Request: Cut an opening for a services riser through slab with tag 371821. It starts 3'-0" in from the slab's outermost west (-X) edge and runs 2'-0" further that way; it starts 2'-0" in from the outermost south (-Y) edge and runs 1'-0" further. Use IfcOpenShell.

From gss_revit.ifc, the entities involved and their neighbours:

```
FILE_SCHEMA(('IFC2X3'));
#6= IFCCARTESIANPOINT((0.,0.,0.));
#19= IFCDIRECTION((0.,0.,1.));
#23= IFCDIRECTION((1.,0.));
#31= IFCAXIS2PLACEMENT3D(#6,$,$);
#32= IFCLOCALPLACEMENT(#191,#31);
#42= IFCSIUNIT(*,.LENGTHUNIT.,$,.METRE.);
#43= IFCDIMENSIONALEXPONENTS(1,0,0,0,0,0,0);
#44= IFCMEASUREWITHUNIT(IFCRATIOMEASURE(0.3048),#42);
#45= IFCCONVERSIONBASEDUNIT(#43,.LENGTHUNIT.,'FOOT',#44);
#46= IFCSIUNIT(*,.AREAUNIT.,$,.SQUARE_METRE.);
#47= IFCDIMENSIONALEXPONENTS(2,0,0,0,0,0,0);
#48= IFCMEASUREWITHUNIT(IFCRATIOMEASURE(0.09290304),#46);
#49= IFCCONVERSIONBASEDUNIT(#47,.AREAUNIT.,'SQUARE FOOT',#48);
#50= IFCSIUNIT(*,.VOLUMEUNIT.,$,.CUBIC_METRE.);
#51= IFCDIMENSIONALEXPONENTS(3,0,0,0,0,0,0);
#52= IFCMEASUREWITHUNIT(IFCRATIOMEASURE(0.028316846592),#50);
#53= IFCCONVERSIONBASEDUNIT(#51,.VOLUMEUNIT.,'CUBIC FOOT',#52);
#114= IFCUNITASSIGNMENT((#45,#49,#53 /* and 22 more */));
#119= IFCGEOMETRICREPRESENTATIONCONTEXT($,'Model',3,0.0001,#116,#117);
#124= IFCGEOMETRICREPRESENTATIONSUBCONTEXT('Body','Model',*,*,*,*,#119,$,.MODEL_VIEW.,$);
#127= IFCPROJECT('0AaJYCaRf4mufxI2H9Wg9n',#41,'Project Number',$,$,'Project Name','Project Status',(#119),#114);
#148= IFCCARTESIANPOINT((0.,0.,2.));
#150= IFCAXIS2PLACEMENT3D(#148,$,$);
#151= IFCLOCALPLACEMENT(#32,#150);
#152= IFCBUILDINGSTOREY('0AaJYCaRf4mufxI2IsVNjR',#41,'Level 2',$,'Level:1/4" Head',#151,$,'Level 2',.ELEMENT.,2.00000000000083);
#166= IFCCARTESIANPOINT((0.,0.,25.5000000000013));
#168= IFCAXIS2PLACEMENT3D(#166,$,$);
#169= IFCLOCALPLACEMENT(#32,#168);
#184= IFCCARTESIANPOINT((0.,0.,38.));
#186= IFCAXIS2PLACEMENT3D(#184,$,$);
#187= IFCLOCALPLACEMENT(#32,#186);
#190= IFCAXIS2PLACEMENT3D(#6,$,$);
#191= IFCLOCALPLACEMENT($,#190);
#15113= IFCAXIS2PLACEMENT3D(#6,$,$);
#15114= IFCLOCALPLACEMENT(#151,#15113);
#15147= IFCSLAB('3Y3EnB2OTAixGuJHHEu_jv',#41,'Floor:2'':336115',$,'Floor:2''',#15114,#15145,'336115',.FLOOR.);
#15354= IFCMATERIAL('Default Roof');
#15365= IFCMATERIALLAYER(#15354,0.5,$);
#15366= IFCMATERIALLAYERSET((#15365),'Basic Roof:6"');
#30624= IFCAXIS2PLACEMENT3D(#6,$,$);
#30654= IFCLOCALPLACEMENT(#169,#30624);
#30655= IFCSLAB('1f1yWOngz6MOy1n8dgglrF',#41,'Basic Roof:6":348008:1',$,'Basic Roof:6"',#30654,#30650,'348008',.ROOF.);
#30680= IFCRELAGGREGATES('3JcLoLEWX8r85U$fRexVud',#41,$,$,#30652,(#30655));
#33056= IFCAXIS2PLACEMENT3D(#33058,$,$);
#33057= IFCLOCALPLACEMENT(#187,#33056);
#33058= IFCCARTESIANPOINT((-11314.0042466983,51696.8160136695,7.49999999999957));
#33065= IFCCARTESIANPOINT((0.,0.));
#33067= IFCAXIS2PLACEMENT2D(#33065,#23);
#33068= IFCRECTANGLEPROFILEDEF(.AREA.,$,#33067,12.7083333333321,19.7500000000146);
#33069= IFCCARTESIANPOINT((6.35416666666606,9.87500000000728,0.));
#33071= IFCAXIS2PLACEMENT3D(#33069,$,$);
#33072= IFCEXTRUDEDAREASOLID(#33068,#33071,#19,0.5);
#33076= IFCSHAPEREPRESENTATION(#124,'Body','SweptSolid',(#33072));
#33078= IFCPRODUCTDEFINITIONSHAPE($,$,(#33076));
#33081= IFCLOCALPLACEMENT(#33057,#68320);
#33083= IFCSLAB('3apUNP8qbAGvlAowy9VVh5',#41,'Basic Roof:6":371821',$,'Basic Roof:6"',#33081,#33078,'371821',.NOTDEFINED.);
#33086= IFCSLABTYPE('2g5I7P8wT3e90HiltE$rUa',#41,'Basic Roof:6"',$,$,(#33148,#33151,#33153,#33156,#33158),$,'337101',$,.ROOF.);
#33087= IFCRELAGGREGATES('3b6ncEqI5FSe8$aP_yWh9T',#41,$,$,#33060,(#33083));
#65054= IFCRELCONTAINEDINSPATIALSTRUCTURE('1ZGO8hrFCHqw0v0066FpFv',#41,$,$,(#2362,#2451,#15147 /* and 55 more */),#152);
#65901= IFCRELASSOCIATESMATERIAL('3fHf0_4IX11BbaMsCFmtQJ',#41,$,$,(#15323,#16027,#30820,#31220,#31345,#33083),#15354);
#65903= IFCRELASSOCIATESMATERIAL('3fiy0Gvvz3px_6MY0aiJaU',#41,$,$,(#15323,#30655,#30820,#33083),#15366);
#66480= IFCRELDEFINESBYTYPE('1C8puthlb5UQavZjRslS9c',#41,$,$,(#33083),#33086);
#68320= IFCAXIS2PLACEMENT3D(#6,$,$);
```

```python
import numpy as np
import ifcopenshell
import ifcopenshell.api.feature
import ifcopenshell.api.geometry
import ifcopenshell.api.root
import ifcopenshell.geom
import ifcopenshell.util.placement
import ifcopenshell.util.representation
import ifcopenshell.util.shape
import ifcopenshell.util.unit

model = ifcopenshell.open("gss_revit.ifc")
unit_scale = ifcopenshell.util.unit.calculate_unit_scale(model)
settings = ifcopenshell.geom.settings()


def volume(element):
    """Net volume in cubic metres, openings subtracted."""
    shape = ifcopenshell.geom.create_shape(settings, element)
    return ifcopenshell.util.shape.get_volume(shape.geometry)


slab = model.by_guid("3apUNP8qbAGvlAowy9VVh5")
before = volume(slab)

# Extent in the slab's own axes, in metres. The edges named are its -X and -Y sides.
slab_shape = ifcopenshell.geom.create_shape(settings, slab)
vertices = ifcopenshell.util.shape.get_vertices(slab_shape.geometry)
x_min, y_min, bottom = vertices.min(axis=0)
top = vertices[:, 2].max()

opening = ifcopenshell.api.root.create_entity(model, ifc_class="IfcOpeningElement", name="Services riser opening")
context = ifcopenshell.util.representation.get_context(model, "Model", "Body", "MODEL_VIEW")
width, depth = 0.6096, 0.3048
outline = [(0.0, 0.0), (width, 0.0), (width, depth), (0.0, depth), (0.0, 0.0)]
# Overshoot both faces by 50 mm so the cut is clean.
shape = ifcopenshell.api.geometry.add_slab_representation(
    model, context=context, depth=top - bottom + 0.1, polyline=outline
)
ifcopenshell.api.geometry.assign_representation(model, product=opening, representation=shape)

matrix = ifcopenshell.util.placement.get_local_placement(slab.ObjectPlacement)
matrix[:, 3] = matrix @ np.append(np.array([x_min + 0.9144, y_min + 0.6096, bottom - 0.05]) / unit_scale, 1.0)
ifcopenshell.api.geometry.edit_object_placement(model, product=opening, matrix=matrix, is_si=False)
ifcopenshell.api.feature.add_feature(model, feature=opening, element=slab)

after = volume(slab)

print(f"slab volume {before:.3f} -> {after:.3f} m3")

model.write("gss_revit-out.ifc")
```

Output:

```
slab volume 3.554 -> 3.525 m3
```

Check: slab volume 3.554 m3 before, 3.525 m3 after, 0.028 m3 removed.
